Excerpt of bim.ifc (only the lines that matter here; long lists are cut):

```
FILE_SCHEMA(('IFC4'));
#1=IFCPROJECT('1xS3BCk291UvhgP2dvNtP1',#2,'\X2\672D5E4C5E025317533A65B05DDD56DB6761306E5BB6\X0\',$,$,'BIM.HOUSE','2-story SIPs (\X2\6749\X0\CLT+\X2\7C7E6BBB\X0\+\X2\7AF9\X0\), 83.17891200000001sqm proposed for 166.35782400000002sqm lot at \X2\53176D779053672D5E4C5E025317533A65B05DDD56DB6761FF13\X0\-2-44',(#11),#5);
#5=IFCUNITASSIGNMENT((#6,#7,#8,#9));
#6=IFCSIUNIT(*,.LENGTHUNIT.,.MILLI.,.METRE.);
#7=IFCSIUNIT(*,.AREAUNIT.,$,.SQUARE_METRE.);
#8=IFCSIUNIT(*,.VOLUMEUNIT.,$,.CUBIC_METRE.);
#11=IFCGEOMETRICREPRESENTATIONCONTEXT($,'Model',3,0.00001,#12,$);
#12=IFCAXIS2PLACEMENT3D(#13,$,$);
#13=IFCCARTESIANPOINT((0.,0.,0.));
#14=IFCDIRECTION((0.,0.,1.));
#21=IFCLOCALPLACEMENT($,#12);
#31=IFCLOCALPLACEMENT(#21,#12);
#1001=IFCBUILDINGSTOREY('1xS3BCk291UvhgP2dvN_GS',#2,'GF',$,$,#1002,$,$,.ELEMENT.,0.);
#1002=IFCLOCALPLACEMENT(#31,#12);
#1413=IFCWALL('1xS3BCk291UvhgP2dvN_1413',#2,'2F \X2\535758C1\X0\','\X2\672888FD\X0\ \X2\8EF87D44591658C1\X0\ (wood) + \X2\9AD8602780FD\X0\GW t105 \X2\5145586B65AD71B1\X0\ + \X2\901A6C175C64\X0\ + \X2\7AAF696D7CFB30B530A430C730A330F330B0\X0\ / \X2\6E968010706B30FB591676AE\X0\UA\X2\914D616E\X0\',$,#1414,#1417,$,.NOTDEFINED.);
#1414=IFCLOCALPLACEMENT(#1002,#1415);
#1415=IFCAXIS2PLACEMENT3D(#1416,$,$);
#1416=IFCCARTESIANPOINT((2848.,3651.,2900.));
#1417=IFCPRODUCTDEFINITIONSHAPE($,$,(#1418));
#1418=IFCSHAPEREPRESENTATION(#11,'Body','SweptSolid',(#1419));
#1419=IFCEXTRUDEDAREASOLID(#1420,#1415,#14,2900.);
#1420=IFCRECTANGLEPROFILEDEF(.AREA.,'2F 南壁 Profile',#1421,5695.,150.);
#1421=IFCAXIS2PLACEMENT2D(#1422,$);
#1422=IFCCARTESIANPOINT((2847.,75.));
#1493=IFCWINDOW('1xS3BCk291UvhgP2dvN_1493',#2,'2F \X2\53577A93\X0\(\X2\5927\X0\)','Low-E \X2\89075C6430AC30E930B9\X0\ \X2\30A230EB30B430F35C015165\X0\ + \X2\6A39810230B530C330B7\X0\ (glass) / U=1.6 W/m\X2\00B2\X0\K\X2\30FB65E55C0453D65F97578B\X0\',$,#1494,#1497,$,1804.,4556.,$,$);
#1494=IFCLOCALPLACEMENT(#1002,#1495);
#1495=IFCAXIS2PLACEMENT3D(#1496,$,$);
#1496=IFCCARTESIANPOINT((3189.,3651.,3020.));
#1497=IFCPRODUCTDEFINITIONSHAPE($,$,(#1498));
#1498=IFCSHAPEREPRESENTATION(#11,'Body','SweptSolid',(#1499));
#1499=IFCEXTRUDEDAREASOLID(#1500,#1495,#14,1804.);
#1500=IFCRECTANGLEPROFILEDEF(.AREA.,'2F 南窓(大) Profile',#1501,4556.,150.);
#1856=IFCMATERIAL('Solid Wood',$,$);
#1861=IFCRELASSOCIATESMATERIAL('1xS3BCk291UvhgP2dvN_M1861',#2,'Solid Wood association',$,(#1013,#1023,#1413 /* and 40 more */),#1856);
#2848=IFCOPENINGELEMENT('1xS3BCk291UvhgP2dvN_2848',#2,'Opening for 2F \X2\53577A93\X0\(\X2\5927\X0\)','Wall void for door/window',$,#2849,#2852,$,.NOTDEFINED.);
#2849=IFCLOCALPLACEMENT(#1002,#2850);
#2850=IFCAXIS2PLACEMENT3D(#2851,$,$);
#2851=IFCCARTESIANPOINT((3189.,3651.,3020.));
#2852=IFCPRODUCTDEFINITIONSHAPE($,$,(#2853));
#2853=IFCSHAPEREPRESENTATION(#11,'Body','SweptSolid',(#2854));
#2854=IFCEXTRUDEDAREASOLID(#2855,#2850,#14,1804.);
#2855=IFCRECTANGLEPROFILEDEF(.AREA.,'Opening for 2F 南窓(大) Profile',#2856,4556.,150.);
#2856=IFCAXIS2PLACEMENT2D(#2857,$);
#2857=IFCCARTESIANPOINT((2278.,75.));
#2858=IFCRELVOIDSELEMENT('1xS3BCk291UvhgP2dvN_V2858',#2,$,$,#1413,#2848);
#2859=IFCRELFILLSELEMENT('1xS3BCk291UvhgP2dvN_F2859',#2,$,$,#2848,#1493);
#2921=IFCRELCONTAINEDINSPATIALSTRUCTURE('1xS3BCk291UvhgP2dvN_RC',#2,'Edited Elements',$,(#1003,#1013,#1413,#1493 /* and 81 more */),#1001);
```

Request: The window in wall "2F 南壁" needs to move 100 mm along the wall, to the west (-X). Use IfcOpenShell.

```python
import ifcopenshell
import ifcopenshell.api.geometry
import ifcopenshell.util.placement

model = ifcopenshell.open("bim.ifc")

window = model.by_guid("1xS3BCk291UvhgP2dvN_1493")
opening = window.FillsVoids[0].RelatingOpeningElement
wall = opening.VoidsElements[0].RelatingBuildingElement

wall_matrix = ifcopenshell.util.placement.get_local_placement(wall.ObjectPlacement)
shift = wall_matrix[:3, 0] * -100.0
before = ifcopenshell.util.placement.get_local_placement(window.ObjectPlacement)[:3, 3].copy()

# The window is not placed relative to its opening, so move both.
for product in (opening, window):
    matrix = ifcopenshell.util.placement.get_local_placement(product.ObjectPlacement)
    matrix[:3, 3] += shift
    ifcopenshell.api.geometry.edit_object_placement(model, product=product, matrix=matrix, is_si=False)

after = ifcopenshell.util.placement.get_local_placement(window.ObjectPlacement)[:3, 3]
print("window moved by", (after - before).round(3) + 0.0)

model.write("bim_updated.ifc")
```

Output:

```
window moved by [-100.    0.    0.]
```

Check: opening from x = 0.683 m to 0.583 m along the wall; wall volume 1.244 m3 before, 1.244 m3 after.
